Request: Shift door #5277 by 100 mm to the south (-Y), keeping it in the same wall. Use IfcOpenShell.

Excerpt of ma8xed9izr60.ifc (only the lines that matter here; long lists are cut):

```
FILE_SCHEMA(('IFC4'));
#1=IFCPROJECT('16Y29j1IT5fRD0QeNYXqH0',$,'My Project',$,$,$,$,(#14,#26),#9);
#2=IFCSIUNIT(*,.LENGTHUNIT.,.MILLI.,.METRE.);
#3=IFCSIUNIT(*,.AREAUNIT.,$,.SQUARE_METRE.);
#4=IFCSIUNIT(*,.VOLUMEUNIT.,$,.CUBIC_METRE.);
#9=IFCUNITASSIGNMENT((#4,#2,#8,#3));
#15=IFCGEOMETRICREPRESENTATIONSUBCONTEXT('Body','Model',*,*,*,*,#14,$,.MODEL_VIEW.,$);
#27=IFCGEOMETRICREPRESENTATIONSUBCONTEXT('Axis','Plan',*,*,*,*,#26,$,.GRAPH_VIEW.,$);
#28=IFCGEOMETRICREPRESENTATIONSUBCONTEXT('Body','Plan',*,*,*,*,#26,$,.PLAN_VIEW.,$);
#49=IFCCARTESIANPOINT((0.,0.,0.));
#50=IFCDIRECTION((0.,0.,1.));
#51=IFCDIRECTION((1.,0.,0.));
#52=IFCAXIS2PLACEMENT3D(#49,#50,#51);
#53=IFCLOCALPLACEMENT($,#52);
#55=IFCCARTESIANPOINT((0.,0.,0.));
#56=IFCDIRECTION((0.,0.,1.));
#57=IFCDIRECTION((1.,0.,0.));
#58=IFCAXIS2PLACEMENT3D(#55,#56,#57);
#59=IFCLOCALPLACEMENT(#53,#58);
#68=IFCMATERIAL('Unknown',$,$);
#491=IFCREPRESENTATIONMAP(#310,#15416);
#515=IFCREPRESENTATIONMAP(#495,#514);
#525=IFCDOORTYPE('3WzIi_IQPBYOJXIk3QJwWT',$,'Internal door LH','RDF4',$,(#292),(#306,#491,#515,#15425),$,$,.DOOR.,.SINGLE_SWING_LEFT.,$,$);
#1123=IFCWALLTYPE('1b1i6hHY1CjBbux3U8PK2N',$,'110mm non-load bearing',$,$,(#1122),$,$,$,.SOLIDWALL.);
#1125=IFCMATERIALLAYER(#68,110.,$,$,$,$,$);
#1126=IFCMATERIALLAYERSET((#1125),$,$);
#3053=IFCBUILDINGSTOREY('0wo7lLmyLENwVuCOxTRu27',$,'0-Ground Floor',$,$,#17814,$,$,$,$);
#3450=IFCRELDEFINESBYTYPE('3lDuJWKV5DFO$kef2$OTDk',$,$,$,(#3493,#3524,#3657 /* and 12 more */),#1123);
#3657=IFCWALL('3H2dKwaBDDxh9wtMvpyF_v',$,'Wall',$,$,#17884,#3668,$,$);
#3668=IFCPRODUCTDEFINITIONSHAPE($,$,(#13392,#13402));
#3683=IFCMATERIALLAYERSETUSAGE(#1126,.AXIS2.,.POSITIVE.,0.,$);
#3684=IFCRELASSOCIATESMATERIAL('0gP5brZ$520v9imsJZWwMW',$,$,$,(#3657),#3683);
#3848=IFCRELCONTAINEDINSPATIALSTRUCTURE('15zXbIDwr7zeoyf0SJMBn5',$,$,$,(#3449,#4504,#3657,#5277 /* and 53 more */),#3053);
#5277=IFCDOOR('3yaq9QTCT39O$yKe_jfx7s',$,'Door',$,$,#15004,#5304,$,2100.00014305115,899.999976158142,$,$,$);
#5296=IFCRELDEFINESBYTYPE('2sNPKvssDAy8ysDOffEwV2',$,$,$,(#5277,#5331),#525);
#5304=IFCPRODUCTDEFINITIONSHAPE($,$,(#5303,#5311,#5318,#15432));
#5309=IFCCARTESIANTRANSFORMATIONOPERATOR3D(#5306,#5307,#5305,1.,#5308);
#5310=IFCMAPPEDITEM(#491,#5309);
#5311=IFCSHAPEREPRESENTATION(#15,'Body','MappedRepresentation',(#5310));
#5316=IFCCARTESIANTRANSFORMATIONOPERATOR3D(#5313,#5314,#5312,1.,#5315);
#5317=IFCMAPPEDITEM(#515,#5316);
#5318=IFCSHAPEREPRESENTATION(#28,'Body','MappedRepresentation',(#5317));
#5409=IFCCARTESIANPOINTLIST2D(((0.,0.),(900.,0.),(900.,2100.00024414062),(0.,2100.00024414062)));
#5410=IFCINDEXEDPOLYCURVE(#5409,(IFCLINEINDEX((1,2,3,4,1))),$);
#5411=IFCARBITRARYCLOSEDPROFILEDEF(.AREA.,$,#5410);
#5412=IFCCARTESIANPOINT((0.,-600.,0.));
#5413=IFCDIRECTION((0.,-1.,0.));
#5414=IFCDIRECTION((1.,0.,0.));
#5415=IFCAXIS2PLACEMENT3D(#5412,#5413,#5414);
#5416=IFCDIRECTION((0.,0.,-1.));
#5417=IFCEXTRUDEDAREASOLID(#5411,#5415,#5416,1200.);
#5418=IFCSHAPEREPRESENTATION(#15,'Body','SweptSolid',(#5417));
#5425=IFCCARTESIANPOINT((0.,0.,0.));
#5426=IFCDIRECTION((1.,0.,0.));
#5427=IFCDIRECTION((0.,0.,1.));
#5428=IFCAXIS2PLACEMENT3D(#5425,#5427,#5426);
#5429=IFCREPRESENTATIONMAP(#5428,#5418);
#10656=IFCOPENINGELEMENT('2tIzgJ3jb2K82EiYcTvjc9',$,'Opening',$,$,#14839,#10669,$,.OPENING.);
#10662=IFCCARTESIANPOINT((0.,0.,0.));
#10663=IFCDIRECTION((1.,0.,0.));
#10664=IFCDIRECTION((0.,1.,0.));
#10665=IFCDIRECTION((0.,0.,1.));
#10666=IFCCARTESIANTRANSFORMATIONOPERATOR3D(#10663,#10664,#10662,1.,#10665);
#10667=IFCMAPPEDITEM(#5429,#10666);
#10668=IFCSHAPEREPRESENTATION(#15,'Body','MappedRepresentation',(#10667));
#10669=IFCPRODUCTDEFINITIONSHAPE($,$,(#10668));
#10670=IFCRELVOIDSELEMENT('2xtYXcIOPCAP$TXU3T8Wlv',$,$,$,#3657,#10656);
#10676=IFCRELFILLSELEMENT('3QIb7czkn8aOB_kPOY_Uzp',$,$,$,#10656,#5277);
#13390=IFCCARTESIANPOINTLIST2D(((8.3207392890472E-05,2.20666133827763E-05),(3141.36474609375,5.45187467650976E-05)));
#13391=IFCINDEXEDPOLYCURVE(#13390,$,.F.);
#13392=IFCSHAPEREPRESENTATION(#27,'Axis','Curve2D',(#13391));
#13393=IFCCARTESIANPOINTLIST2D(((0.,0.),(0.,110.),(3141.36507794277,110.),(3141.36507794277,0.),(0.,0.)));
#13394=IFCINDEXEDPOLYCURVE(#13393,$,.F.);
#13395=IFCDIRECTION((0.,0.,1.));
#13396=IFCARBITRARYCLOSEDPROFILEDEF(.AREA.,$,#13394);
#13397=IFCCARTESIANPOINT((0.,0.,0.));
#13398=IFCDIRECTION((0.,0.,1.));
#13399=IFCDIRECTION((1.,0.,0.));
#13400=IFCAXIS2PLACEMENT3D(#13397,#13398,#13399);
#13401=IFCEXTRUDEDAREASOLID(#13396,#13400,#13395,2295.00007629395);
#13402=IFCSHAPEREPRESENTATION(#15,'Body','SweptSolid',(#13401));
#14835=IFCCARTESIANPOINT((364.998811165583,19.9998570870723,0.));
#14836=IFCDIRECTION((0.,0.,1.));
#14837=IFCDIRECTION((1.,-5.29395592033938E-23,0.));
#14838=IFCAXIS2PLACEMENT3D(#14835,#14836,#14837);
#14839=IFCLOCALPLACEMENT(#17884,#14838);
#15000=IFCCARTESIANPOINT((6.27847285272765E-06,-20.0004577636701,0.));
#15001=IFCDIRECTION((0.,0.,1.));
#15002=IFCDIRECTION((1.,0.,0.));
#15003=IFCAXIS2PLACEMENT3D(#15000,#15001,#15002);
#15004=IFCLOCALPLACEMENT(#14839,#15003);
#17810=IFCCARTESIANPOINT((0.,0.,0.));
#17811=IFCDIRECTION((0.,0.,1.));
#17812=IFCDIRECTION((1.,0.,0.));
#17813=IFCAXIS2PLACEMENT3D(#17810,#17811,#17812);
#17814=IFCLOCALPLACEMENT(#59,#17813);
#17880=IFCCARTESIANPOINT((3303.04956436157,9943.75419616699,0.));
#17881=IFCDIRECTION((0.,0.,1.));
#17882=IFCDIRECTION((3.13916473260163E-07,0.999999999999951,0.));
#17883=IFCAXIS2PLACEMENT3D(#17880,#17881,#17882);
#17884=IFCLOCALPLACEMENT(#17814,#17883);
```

```python
import ifcopenshell
import ifcopenshell.api.geometry
import ifcopenshell.util.placement
import ifcopenshell.util.unit

model = ifcopenshell.open("ma8xed9izr60.ifc")
unit_scale = ifcopenshell.util.unit.calculate_unit_scale(model)

door = model.by_guid("3yaq9QTCT39O$yKe_jfx7s")
opening = door.FillsVoids[0].RelatingOpeningElement
wall = opening.VoidsElements[0].RelatingBuildingElement

wall_matrix = ifcopenshell.util.placement.get_local_placement(wall.ObjectPlacement)
shift = wall_matrix[:3, 0] * -0.1 / unit_scale
before = ifcopenshell.util.placement.get_local_placement(door.ObjectPlacement)[:3, 3].copy()

# The door is placed relative to its opening, so it follows when the opening moves.
matrix = ifcopenshell.util.placement.get_local_placement(opening.ObjectPlacement)
matrix[:3, 3] += shift
ifcopenshell.api.geometry.edit_object_placement(
    model, product=opening, matrix=matrix, is_si=False, should_transform_children=True
)

after = ifcopenshell.util.placement.get_local_placement(door.ObjectPlacement)[:3, 3]
print("door moved by", (after - before).round(3) + 0.0)

model.write("ma8xed9izr60_updated.ifc")
```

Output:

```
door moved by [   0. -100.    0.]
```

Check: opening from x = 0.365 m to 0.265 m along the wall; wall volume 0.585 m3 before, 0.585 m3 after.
